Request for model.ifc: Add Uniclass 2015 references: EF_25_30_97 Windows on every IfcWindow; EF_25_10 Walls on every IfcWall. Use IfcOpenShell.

First a look at what the model holds.

```python
import ifcopenshell

model = ifcopenshell.open("model.ifc")
print(model.schema)
print("classifications:", [c.Name for c in model.by_type("IfcClassification")])
for ifc_class in ("IfcDoor", "IfcRoof", "IfcStair", "IfcWall", "IfcWindow"):
    print(ifc_class, len(model.by_type(ifc_class)))
```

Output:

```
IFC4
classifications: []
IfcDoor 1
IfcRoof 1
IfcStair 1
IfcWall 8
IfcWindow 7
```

```python
import ifcopenshell
import ifcopenshell.api.classification

model = ifcopenshell.open("model.ifc")

system = ifcopenshell.api.classification.add_classification(model, classification="Uniclass 2015")

codes = {
    "IfcWindow": ("EF_25_30_97", "Windows"),
    "IfcWall": ("EF_25_10", "Walls"),
}
for ifc_class, (code, name) in codes.items():
    products = model.by_type(ifc_class)
    ifcopenshell.api.classification.add_reference(
        model, products=products, classification=system, identification=code, name=name
    )
    print(code, len(products))

model.write("model_updated.ifc")
```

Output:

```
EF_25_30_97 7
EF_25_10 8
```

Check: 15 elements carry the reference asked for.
